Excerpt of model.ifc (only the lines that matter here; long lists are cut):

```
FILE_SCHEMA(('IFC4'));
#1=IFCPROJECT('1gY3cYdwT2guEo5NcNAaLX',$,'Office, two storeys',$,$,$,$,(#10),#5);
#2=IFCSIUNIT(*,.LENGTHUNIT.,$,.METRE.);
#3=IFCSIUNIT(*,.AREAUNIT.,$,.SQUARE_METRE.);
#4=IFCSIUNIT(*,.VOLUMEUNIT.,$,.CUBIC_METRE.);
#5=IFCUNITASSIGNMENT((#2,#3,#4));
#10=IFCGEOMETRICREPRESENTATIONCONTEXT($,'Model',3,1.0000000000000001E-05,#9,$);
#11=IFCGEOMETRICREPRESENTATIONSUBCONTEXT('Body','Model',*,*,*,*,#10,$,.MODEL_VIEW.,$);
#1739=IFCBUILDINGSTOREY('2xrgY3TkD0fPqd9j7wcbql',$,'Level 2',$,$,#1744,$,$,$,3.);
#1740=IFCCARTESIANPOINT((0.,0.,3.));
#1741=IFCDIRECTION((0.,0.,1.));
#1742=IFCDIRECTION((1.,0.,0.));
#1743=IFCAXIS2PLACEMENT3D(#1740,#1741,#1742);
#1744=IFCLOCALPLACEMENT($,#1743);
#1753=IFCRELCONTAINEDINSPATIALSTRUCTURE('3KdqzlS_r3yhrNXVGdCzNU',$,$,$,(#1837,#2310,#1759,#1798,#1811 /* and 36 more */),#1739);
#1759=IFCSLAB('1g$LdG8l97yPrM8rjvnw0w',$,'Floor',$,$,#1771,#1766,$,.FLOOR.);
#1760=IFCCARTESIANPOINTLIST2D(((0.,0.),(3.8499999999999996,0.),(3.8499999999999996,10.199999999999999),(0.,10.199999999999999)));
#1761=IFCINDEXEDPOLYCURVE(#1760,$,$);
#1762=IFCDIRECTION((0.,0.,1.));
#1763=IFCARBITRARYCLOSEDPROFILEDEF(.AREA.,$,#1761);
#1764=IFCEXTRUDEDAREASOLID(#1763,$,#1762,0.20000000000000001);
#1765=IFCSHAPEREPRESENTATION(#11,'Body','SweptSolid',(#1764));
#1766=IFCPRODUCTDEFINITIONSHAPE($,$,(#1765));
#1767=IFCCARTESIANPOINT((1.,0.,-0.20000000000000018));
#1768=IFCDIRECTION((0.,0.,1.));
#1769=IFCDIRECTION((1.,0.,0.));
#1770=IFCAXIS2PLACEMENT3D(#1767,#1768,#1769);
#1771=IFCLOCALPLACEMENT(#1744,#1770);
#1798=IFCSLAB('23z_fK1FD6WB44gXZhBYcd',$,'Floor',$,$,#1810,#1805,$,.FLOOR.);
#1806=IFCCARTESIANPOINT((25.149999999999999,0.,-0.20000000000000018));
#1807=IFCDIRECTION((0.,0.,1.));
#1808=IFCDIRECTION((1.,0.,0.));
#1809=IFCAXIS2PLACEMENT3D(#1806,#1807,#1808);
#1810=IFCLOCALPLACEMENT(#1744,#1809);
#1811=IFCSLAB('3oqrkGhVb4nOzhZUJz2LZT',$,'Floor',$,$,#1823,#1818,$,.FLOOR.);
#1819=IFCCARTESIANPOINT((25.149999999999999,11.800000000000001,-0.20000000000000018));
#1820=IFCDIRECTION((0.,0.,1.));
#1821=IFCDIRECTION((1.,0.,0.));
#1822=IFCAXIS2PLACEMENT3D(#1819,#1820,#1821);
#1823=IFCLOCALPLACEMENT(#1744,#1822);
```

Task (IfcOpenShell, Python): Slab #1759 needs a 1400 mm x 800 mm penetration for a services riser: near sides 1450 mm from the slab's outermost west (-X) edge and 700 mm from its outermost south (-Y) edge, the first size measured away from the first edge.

```python
import numpy as np
import ifcopenshell
import ifcopenshell.api.feature
import ifcopenshell.api.geometry
import ifcopenshell.api.root
import ifcopenshell.geom
import ifcopenshell.util.placement
import ifcopenshell.util.representation
import ifcopenshell.util.shape
import ifcopenshell.util.unit

model = ifcopenshell.open("model.ifc")
unit_scale = ifcopenshell.util.unit.calculate_unit_scale(model)
settings = ifcopenshell.geom.settings()


def volume(element):
    """Net volume in cubic metres, openings subtracted."""
    shape = ifcopenshell.geom.create_shape(settings, element)
    return ifcopenshell.util.shape.get_volume(shape.geometry)


slab = model.by_guid("1g$LdG8l97yPrM8rjvnw0w")
before = volume(slab)

# Extent in the slab's own axes, in metres. The edges named are its -X and -Y sides.
slab_shape = ifcopenshell.geom.create_shape(settings, slab)
vertices = ifcopenshell.util.shape.get_vertices(slab_shape.geometry)
x_min, y_min, bottom = vertices.min(axis=0)
top = vertices[:, 2].max()

opening = ifcopenshell.api.root.create_entity(model, ifc_class="IfcOpeningElement", name="Services riser opening", predefined_type="OPENING")
context = ifcopenshell.util.representation.get_context(model, "Model", "Body", "MODEL_VIEW")
width, depth = 1.4, 0.8
outline = [(0.0, 0.0), (width, 0.0), (width, depth), (0.0, depth), (0.0, 0.0)]
# Overshoot both faces by 50 mm so the cut is clean.
shape = ifcopenshell.api.geometry.add_slab_representation(
    model, context=context, depth=top - bottom + 0.1, polyline=outline
)
ifcopenshell.api.geometry.assign_representation(model, product=opening, representation=shape)

matrix = ifcopenshell.util.placement.get_local_placement(slab.ObjectPlacement)
matrix[:, 3] = matrix @ np.append(np.array([x_min + 1.45, y_min + 0.7, bottom - 0.05]) / unit_scale, 1.0)
ifcopenshell.api.geometry.edit_object_placement(model, product=opening, matrix=matrix, is_si=False)
ifcopenshell.api.feature.add_feature(model, feature=opening, element=slab)

after = volume(slab)

print(f"slab volume {before:.3f} -> {after:.3f} m3")

model.write("model_v2.ifc")
```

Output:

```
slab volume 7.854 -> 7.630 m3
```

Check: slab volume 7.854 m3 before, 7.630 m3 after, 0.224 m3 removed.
